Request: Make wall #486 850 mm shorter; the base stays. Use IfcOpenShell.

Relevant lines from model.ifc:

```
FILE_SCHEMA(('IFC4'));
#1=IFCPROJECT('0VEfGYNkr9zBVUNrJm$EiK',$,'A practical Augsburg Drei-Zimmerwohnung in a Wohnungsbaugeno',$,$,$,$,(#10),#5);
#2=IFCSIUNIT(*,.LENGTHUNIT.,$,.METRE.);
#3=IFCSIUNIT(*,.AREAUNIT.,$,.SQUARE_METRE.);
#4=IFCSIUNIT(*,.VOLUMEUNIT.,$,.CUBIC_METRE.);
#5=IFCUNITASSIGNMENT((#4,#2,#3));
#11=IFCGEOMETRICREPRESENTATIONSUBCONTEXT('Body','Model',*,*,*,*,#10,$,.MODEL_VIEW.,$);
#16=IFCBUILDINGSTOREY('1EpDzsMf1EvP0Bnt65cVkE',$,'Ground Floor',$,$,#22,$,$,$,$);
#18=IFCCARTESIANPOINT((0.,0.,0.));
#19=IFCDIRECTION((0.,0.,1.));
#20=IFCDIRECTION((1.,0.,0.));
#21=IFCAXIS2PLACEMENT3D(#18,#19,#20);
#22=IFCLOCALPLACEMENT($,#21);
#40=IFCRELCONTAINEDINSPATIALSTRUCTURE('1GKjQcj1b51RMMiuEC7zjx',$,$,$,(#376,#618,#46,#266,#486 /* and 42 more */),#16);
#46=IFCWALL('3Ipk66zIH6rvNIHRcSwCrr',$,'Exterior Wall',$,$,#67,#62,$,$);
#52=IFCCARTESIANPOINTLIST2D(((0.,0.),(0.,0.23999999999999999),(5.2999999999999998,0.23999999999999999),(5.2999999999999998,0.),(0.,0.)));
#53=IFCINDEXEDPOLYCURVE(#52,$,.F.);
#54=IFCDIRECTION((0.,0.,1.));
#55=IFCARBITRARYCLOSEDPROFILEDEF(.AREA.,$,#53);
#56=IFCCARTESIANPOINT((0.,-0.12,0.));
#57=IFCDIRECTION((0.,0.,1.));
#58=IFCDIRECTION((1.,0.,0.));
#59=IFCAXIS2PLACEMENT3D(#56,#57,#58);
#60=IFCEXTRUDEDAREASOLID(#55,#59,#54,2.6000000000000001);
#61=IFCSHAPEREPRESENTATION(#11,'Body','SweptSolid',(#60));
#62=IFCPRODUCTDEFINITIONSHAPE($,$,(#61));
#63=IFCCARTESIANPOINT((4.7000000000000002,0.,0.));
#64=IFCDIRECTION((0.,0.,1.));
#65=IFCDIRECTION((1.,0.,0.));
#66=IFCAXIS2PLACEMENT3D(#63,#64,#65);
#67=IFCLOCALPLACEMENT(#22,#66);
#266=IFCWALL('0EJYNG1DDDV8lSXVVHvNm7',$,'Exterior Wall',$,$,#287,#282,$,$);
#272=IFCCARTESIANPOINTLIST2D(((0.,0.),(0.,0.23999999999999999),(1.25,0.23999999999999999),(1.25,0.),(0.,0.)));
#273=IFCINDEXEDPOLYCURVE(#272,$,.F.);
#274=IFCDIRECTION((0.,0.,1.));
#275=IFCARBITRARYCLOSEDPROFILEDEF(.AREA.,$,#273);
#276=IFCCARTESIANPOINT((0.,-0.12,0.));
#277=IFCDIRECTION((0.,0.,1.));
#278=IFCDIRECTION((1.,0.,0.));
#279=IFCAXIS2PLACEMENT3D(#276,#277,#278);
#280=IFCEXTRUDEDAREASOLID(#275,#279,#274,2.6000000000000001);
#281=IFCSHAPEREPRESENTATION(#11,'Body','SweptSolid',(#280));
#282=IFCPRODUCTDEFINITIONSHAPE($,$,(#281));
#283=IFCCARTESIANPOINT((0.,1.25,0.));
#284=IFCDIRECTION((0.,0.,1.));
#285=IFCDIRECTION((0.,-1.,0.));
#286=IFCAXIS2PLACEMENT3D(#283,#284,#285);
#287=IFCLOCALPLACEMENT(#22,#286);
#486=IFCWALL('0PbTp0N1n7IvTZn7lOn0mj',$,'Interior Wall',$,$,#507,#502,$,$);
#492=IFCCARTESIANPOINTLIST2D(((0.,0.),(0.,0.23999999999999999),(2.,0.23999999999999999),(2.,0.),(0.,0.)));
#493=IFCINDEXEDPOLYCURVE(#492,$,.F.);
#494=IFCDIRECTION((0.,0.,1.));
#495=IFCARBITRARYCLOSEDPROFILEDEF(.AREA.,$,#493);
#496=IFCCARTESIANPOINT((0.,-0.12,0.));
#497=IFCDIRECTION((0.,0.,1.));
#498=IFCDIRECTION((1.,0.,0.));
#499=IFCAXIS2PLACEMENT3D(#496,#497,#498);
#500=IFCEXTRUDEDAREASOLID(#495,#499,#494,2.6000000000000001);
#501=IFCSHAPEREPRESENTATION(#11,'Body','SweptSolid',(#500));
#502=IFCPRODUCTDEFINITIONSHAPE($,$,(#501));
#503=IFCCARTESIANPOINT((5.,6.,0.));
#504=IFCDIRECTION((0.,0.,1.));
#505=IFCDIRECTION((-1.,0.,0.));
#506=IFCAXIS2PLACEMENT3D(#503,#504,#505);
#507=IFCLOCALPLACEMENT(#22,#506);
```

```python
import ifcopenshell
import ifcopenshell.geom
import ifcopenshell.util.representation
import ifcopenshell.util.shape
import ifcopenshell.util.unit

model = ifcopenshell.open("model.ifc")
unit_scale = ifcopenshell.util.unit.calculate_unit_scale(model)
settings = ifcopenshell.geom.settings()


def volume(element):
    """Net volume in cubic metres, openings subtracted."""
    shape = ifcopenshell.geom.create_shape(settings, element)
    return ifcopenshell.util.shape.get_volume(shape.geometry)


wall = model.by_id(486)
before = volume(wall)

body = ifcopenshell.util.representation.get_representation(wall, "Model", "Body")
solid = body.Items[0]
old_height = solid.Depth
solid.Depth -= 0.85 / unit_scale
after = volume(wall)

print(f"height {old_height:g} -> {solid.Depth:g}, volume {before:.3f} -> {after:.3f} m3")

model.write("model_rev.ifc")
```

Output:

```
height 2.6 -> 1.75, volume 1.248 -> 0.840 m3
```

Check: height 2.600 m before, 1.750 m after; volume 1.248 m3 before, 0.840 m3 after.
